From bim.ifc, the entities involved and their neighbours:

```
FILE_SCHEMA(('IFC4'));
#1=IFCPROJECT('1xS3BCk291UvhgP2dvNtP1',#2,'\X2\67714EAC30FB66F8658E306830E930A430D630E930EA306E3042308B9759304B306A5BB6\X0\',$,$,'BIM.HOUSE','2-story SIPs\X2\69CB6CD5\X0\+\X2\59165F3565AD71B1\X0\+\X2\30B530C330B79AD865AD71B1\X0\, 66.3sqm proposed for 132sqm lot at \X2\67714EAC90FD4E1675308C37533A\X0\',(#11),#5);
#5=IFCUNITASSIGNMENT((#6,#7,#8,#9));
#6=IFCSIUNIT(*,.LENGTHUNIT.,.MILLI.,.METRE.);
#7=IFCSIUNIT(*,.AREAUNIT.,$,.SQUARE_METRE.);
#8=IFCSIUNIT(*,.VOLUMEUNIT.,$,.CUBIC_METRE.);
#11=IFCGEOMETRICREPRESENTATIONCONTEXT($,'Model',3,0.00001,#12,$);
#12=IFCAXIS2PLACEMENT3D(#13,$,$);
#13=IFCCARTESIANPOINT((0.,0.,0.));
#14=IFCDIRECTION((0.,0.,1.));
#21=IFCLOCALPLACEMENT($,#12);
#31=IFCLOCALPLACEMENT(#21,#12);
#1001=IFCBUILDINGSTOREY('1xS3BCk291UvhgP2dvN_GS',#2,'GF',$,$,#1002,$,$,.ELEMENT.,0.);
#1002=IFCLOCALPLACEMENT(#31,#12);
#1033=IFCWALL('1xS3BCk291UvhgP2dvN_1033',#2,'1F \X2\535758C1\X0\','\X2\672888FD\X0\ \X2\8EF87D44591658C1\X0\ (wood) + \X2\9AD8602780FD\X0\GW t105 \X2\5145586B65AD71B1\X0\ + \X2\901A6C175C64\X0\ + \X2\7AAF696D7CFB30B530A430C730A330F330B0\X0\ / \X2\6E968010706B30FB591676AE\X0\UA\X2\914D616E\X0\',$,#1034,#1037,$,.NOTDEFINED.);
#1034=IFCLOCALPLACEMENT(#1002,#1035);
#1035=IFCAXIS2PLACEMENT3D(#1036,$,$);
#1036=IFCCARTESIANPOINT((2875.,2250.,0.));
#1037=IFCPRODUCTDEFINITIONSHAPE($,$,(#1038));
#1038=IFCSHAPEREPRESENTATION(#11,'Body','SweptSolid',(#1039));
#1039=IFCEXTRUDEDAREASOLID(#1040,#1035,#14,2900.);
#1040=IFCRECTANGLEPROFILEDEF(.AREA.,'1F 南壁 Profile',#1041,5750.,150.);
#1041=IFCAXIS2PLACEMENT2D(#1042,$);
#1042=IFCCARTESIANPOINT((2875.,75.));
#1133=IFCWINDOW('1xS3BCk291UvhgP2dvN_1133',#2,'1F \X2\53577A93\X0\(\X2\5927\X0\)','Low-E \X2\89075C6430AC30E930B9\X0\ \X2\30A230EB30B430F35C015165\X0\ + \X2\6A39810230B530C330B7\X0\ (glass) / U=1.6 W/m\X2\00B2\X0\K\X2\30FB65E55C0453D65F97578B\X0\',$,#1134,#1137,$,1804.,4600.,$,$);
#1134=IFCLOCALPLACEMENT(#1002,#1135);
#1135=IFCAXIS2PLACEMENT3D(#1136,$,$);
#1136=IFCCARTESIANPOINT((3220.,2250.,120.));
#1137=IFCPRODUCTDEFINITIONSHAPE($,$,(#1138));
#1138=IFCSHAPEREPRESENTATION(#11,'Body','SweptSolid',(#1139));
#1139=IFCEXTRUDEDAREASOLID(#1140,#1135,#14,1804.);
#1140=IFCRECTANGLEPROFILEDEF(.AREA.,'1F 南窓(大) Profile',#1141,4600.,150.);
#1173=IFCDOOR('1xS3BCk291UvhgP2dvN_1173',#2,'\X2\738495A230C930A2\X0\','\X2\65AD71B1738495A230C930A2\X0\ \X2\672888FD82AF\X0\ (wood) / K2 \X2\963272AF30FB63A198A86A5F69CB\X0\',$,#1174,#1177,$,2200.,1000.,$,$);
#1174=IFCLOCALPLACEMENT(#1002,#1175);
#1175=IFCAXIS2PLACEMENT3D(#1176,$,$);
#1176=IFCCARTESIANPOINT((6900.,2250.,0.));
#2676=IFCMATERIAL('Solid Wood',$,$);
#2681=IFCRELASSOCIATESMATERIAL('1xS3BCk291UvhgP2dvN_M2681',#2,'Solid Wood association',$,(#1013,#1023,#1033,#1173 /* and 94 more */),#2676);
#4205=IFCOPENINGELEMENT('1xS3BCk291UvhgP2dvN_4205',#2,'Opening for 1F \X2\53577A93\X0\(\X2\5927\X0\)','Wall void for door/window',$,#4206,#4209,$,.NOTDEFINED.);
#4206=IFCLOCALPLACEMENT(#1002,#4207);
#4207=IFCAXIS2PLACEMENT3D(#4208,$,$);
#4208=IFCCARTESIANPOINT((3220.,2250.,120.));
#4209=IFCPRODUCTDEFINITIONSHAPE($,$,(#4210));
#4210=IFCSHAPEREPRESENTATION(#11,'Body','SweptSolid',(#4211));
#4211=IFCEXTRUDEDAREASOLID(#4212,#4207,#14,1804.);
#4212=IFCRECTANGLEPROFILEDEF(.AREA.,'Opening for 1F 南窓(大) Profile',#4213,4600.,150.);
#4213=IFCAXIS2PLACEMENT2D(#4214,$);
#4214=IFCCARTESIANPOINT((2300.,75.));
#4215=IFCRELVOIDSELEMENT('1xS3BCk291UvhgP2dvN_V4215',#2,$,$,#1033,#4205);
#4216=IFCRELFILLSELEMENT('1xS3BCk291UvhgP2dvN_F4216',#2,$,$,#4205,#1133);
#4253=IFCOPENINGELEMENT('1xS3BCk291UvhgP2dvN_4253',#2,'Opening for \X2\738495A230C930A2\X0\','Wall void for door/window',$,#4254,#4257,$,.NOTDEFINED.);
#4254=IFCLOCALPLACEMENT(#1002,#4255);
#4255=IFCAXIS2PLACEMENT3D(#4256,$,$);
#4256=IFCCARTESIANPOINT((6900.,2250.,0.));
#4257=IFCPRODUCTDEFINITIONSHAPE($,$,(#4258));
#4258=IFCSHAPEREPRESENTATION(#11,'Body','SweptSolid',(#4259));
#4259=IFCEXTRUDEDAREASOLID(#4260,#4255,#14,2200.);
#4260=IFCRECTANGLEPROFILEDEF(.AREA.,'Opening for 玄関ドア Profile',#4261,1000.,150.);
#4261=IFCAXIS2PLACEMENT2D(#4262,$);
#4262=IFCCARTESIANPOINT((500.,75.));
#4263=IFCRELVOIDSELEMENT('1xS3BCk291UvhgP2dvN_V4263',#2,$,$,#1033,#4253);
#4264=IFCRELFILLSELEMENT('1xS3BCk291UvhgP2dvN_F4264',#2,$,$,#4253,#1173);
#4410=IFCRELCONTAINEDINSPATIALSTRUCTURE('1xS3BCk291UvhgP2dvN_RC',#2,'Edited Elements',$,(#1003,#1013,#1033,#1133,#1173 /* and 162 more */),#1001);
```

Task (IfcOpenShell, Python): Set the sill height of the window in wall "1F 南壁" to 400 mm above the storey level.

```python
import numpy as np
import ifcopenshell
import ifcopenshell.api.geometry
import ifcopenshell.geom
import ifcopenshell.util.element
import ifcopenshell.util.placement
import ifcopenshell.util.shape
import ifcopenshell.util.unit

model = ifcopenshell.open("bim.ifc")
unit_scale = ifcopenshell.util.unit.calculate_unit_scale(model)

window = model.by_id(1133)
opening = window.FillsVoids[0].RelatingOpeningElement
storey = ifcopenshell.util.element.get_container(window, ifc_class="IfcBuildingStorey")
level = ifcopenshell.util.placement.get_local_placement(storey.ObjectPlacement)[2, 3]

# The opening's origin need not be at the sill, so measure its lowest point.
shape = ifcopenshell.geom.create_shape(ifcopenshell.geom.settings(), opening)
bottom = ifcopenshell.util.shape.get_shape_bottom_elevation(shape, shape.geometry) / unit_scale
dz = level + 0.4 / unit_scale - bottom

shift = np.array([0.0, 0.0, dz])
# The window is not placed relative to its opening, so move both.
for product in (opening, window):
    matrix = ifcopenshell.util.placement.get_local_placement(product.ObjectPlacement)
    matrix[:3, 3] += shift
    ifcopenshell.api.geometry.edit_object_placement(model, product=product, matrix=matrix, is_si=False)

print(f"moved by {dz * unit_scale:+.3f} m")

model.write("bim_edited.ifc")
```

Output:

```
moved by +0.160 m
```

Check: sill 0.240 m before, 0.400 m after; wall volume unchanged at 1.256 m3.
